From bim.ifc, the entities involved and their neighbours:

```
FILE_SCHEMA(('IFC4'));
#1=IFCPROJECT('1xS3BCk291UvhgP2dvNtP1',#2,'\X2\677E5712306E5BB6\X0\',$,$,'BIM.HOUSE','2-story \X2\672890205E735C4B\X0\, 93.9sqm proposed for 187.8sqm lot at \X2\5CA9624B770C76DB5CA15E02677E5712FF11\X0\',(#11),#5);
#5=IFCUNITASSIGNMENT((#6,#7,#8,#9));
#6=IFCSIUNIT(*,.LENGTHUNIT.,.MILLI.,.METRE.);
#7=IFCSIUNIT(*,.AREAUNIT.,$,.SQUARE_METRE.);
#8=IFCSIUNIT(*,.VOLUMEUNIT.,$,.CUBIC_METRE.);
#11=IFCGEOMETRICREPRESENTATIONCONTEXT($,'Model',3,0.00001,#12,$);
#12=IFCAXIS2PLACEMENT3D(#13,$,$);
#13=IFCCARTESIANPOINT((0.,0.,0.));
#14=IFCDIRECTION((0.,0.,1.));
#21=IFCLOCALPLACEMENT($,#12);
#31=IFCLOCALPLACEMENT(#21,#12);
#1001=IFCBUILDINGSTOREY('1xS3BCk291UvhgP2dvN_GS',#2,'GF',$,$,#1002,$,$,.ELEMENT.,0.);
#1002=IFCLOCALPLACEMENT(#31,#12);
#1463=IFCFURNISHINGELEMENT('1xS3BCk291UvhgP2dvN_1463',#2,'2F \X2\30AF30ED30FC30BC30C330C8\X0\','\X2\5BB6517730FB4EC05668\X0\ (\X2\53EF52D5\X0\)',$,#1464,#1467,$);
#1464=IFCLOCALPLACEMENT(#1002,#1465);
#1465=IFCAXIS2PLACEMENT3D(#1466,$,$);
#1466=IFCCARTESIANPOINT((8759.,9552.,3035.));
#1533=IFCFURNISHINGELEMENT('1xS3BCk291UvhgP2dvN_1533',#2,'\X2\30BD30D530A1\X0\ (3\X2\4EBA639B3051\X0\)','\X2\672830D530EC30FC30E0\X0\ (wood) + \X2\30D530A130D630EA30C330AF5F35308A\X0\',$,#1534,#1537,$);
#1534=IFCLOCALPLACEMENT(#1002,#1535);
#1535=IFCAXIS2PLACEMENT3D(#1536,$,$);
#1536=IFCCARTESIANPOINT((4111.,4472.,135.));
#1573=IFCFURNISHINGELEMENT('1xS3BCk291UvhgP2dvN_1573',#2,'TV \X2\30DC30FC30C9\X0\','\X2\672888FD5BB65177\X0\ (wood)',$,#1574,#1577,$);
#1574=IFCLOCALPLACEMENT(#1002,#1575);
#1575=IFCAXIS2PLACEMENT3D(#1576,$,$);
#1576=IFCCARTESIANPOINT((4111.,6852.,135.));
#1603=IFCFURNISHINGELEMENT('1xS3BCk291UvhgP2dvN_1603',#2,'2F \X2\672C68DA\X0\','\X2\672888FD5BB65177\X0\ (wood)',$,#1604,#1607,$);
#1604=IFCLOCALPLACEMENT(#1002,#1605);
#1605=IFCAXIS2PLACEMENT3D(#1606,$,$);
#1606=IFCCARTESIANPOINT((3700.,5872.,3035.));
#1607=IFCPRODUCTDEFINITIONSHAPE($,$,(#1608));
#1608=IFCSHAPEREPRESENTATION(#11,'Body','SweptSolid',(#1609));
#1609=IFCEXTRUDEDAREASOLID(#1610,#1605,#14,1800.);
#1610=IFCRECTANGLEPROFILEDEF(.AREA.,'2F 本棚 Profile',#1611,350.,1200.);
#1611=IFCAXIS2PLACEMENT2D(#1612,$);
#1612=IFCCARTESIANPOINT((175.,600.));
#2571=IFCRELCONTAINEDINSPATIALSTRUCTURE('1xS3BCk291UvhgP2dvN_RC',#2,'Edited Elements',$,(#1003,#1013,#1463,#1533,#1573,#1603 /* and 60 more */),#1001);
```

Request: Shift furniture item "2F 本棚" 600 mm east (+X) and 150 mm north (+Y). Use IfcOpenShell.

```python
import ifcopenshell
import ifcopenshell.api.geometry
import ifcopenshell.util.placement
import ifcopenshell.util.unit

model = ifcopenshell.open("bim.ifc")
unit_scale = ifcopenshell.util.unit.calculate_unit_scale(model)

item = model.by_guid("1xS3BCk291UvhgP2dvN_1603")
matrix = ifcopenshell.util.placement.get_local_placement(item.ObjectPlacement)
matrix[0, 3] += 0.6 / unit_scale
matrix[1, 3] += 0.15 / unit_scale
ifcopenshell.api.geometry.edit_object_placement(model, product=item, matrix=matrix, is_si=False)

print(ifcopenshell.util.placement.get_local_placement(item.ObjectPlacement).round(3) + 0.0)

model.write("bim_v2.ifc")
```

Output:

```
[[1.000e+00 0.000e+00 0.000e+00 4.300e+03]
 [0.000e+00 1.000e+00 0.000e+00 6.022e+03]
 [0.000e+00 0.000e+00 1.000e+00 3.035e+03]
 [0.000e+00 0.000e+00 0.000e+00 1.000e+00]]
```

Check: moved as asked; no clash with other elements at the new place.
